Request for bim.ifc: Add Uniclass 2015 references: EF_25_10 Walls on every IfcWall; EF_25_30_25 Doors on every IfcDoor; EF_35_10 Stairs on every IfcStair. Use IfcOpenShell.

First a look at what the model holds.

```python
import ifcopenshell

model = ifcopenshell.open("bim.ifc")
print(model.schema)
print("classifications:", [c.Name for c in model.by_type("IfcClassification")])
for ifc_class in ("IfcDoor", "IfcRoof", "IfcStair", "IfcWall", "IfcWindow"):
    print(ifc_class, len(model.by_type(ifc_class)))
```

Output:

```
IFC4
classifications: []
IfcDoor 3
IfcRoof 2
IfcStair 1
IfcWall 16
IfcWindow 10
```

```python
import ifcopenshell
import ifcopenshell.api.classification

model = ifcopenshell.open("bim.ifc")

system = ifcopenshell.api.classification.add_classification(model, classification="Uniclass 2015")

codes = {
    "IfcWall": ("EF_25_10", "Walls"),
    "IfcDoor": ("EF_25_30_25", "Doors"),
    "IfcStair": ("EF_35_10", "Stairs"),
}
for ifc_class, (code, name) in codes.items():
    products = model.by_type(ifc_class)
    ifcopenshell.api.classification.add_reference(
        model, products=products, classification=system, identification=code, name=name
    )
    print(code, len(products))

model.write("bim_updated.ifc")
```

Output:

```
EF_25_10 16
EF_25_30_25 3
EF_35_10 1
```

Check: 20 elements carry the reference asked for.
